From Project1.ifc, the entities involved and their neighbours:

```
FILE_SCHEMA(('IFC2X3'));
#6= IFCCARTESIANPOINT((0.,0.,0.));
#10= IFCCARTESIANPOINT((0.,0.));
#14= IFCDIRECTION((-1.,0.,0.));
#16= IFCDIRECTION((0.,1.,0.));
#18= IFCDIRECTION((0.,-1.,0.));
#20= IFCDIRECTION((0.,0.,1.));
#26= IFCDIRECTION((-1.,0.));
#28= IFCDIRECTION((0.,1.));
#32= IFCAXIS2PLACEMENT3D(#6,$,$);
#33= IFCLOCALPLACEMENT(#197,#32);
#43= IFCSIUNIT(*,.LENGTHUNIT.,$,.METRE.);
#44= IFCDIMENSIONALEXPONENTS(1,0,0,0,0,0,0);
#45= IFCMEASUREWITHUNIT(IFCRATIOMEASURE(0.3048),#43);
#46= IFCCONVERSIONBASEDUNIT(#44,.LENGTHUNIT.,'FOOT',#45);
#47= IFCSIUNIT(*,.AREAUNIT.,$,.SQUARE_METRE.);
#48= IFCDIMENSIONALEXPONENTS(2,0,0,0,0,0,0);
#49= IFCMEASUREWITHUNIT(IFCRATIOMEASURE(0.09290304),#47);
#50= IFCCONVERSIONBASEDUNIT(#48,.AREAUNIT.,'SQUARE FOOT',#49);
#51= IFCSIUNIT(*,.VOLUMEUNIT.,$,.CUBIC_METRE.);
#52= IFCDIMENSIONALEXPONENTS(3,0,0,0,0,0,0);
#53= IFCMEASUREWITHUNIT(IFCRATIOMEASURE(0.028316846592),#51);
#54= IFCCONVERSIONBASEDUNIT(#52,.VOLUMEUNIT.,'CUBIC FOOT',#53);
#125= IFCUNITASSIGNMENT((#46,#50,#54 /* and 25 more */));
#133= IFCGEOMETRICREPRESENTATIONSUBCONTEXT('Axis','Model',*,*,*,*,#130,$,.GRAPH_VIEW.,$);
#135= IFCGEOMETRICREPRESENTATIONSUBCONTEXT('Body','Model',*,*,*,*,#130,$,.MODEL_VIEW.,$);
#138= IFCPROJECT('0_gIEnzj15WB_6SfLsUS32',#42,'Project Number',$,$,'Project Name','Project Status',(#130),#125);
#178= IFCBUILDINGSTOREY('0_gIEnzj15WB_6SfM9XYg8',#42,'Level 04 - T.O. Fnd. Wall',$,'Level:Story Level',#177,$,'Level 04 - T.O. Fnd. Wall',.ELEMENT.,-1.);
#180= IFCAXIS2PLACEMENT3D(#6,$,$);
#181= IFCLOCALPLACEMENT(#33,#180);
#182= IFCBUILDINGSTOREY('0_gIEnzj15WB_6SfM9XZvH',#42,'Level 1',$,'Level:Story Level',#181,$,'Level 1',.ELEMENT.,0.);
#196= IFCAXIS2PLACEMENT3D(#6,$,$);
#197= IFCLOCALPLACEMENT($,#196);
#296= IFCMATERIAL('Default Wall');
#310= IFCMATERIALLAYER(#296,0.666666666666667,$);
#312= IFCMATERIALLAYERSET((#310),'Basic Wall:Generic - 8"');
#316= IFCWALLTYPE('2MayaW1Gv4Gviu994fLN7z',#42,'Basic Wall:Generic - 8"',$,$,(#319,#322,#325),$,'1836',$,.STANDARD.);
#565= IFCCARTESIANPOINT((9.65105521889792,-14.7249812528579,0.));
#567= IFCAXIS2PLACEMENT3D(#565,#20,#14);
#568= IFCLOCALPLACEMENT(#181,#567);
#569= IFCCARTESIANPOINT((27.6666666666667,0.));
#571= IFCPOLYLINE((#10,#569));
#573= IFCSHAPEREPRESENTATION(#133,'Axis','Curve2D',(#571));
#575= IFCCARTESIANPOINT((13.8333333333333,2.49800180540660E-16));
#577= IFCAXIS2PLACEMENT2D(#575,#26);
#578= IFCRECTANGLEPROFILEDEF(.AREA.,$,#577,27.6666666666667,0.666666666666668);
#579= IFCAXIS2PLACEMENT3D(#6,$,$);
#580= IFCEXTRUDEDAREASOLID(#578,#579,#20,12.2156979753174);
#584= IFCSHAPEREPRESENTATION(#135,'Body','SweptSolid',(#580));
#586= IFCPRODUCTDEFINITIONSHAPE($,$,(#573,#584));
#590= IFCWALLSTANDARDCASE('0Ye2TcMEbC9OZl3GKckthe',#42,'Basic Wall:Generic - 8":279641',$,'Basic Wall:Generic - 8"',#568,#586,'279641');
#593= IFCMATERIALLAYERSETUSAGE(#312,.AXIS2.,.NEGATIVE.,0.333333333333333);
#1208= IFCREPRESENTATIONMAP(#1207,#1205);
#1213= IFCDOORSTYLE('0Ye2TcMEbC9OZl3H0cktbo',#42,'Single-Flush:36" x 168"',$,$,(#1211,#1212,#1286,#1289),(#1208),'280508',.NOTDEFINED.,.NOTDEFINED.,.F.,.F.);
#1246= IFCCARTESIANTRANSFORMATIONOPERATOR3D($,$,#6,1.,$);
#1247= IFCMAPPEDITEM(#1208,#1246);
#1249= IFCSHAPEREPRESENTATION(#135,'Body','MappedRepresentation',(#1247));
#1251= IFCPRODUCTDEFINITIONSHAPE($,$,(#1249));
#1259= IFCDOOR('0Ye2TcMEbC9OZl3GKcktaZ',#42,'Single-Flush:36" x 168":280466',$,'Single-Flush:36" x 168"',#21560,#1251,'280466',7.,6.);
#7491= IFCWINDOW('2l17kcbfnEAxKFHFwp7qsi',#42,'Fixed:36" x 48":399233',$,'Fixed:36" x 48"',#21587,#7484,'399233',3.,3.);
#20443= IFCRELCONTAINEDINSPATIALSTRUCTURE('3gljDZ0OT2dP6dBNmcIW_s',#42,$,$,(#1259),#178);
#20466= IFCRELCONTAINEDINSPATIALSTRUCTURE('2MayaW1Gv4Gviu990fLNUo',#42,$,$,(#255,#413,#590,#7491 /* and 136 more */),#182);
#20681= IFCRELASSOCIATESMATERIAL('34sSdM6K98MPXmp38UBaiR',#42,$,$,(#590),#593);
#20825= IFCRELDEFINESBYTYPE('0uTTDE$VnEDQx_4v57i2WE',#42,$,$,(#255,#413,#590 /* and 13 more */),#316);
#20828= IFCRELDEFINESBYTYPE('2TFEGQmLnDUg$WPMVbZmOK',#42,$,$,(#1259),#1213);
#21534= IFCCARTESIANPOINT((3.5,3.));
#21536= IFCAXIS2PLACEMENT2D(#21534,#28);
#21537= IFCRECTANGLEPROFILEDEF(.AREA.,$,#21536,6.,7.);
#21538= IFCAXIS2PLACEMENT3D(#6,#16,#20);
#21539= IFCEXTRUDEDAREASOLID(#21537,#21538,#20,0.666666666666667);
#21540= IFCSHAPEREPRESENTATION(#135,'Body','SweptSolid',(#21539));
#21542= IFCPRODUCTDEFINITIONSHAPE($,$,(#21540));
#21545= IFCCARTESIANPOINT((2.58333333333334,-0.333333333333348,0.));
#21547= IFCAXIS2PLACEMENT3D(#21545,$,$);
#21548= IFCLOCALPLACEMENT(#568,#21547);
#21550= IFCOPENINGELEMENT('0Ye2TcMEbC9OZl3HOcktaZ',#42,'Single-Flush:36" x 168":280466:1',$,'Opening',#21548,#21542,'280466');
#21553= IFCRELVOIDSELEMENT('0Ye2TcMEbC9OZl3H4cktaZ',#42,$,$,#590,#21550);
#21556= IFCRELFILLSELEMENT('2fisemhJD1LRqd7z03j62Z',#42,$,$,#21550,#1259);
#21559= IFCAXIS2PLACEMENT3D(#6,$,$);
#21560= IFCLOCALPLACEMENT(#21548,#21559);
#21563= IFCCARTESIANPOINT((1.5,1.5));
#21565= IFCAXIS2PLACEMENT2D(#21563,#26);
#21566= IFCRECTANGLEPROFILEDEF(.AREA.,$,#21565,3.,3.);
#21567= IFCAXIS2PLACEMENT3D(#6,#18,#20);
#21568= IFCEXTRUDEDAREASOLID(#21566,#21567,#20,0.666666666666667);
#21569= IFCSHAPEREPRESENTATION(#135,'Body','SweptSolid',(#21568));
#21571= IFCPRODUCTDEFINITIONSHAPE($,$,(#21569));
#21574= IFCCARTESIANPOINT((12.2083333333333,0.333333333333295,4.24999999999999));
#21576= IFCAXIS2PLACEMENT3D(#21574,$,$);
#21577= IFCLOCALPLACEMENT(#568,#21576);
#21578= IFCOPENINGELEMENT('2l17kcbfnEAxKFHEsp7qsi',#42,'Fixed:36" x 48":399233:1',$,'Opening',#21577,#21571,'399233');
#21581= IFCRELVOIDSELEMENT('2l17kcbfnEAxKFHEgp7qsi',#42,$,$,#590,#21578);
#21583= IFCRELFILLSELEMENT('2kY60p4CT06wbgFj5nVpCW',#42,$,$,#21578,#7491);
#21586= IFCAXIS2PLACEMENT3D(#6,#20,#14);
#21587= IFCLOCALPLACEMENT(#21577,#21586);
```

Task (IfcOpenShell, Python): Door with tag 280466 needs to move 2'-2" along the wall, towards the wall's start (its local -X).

```python
import ifcopenshell
import ifcopenshell.api.geometry
import ifcopenshell.util.placement
import ifcopenshell.util.unit

model = ifcopenshell.open("Project1.ifc")
unit_scale = ifcopenshell.util.unit.calculate_unit_scale(model)

door = model.by_guid("0Ye2TcMEbC9OZl3GKcktaZ")
opening = door.FillsVoids[0].RelatingOpeningElement
wall = opening.VoidsElements[0].RelatingBuildingElement

wall_matrix = ifcopenshell.util.placement.get_local_placement(wall.ObjectPlacement)
shift = wall_matrix[:3, 0] * -26 * 0.0254 / unit_scale
before = ifcopenshell.util.placement.get_local_placement(door.ObjectPlacement)[:3, 3].copy()

# The door is placed relative to its opening, so it follows when the opening moves.
matrix = ifcopenshell.util.placement.get_local_placement(opening.ObjectPlacement)
matrix[:3, 3] += shift
ifcopenshell.api.geometry.edit_object_placement(
    model, product=opening, matrix=matrix, is_si=False, should_transform_children=True
)

after = ifcopenshell.util.placement.get_local_placement(door.ObjectPlacement)[:3, 3]
print("door moved by", (after - before).round(3) + 0.0)

model.write("Project1_updated.ifc")
```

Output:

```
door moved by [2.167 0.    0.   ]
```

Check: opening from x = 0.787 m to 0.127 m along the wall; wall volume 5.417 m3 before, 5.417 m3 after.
